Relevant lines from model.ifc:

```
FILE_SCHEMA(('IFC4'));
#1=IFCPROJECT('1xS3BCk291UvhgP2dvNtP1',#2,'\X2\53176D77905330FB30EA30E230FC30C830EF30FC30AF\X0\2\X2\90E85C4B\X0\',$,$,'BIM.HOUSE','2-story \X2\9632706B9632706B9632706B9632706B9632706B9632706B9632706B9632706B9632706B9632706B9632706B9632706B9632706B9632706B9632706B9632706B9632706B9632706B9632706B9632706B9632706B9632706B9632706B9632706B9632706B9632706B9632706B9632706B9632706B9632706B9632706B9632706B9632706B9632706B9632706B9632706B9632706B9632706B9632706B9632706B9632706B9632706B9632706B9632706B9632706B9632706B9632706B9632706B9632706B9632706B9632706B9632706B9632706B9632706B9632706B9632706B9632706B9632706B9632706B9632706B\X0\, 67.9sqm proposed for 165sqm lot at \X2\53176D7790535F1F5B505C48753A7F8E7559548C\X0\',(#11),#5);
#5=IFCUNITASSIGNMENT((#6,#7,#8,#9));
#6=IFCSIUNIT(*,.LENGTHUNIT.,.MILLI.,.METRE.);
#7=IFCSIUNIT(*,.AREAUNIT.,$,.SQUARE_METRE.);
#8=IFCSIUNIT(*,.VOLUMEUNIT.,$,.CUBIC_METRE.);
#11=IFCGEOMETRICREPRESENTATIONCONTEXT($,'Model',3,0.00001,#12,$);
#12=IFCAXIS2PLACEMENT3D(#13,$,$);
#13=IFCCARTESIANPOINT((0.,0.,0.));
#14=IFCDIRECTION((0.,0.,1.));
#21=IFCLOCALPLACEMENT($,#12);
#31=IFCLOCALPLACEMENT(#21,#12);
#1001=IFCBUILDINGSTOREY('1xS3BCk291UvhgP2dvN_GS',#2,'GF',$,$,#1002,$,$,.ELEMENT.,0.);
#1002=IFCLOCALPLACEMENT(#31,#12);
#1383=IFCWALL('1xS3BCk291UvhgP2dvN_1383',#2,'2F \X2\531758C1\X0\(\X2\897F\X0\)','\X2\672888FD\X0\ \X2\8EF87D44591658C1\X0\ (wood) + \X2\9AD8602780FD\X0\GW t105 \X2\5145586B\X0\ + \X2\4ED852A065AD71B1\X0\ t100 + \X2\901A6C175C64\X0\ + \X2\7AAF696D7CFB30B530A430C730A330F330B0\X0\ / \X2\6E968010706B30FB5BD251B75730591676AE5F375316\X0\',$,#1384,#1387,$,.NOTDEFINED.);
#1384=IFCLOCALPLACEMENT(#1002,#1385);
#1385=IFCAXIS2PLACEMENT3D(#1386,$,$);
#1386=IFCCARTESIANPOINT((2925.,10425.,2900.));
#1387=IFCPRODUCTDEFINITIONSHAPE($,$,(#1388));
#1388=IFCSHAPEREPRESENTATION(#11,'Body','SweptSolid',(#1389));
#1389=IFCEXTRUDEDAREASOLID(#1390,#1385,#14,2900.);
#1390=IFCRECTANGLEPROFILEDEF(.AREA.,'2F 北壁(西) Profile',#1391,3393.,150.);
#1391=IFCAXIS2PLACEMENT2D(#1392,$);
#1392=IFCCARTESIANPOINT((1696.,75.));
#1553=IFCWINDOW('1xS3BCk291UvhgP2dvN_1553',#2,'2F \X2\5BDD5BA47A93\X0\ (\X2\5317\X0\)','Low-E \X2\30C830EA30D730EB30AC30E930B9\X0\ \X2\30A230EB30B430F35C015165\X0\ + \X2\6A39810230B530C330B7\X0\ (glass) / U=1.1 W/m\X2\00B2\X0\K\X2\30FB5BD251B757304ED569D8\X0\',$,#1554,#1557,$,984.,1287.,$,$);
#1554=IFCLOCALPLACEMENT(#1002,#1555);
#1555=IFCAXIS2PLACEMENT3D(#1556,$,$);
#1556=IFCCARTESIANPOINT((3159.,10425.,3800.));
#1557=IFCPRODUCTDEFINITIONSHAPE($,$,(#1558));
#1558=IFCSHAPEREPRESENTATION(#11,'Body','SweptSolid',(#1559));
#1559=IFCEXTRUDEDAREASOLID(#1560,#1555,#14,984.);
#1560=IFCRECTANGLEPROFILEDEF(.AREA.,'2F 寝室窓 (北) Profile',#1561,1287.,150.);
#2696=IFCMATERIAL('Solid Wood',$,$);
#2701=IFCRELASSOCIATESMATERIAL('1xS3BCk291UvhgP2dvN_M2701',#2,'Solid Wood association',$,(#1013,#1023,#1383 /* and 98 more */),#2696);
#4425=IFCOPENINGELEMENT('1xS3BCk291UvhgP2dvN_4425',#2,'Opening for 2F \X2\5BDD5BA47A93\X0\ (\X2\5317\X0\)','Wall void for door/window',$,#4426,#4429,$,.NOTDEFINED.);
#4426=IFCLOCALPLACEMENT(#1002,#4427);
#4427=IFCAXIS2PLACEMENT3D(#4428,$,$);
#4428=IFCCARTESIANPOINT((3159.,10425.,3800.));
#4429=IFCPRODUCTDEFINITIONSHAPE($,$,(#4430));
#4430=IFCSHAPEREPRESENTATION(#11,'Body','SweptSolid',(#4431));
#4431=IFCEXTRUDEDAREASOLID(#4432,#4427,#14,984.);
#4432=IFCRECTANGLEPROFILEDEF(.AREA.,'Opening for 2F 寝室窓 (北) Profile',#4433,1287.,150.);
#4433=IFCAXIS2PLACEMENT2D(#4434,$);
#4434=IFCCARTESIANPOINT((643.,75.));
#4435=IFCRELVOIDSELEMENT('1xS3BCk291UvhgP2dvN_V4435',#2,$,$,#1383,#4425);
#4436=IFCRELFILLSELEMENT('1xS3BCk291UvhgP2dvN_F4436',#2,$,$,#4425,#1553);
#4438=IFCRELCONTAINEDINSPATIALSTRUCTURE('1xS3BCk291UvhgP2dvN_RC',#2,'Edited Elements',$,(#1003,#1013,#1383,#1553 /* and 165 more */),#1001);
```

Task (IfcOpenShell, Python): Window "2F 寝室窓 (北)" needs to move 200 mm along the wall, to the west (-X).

```python
import ifcopenshell
import ifcopenshell.api.geometry
import ifcopenshell.util.placement

model = ifcopenshell.open("model.ifc")

window = model.by_guid("1xS3BCk291UvhgP2dvN_1553")
opening = window.FillsVoids[0].RelatingOpeningElement
wall = opening.VoidsElements[0].RelatingBuildingElement

wall_matrix = ifcopenshell.util.placement.get_local_placement(wall.ObjectPlacement)
shift = wall_matrix[:3, 0] * -200.0
before = ifcopenshell.util.placement.get_local_placement(window.ObjectPlacement)[:3, 3].copy()

# The window is not placed relative to its opening, so move both.
for product in (opening, window):
    matrix = ifcopenshell.util.placement.get_local_placement(product.ObjectPlacement)
    matrix[:3, 3] += shift
    ifcopenshell.api.geometry.edit_object_placement(model, product=product, matrix=matrix, is_si=False)

after = ifcopenshell.util.placement.get_local_placement(window.ObjectPlacement)[:3, 3]
print("window moved by", (after - before).round(3) + 0.0)

model.write("model_rev.ifc")
```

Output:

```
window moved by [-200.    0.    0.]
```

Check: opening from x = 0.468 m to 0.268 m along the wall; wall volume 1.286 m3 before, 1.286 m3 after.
